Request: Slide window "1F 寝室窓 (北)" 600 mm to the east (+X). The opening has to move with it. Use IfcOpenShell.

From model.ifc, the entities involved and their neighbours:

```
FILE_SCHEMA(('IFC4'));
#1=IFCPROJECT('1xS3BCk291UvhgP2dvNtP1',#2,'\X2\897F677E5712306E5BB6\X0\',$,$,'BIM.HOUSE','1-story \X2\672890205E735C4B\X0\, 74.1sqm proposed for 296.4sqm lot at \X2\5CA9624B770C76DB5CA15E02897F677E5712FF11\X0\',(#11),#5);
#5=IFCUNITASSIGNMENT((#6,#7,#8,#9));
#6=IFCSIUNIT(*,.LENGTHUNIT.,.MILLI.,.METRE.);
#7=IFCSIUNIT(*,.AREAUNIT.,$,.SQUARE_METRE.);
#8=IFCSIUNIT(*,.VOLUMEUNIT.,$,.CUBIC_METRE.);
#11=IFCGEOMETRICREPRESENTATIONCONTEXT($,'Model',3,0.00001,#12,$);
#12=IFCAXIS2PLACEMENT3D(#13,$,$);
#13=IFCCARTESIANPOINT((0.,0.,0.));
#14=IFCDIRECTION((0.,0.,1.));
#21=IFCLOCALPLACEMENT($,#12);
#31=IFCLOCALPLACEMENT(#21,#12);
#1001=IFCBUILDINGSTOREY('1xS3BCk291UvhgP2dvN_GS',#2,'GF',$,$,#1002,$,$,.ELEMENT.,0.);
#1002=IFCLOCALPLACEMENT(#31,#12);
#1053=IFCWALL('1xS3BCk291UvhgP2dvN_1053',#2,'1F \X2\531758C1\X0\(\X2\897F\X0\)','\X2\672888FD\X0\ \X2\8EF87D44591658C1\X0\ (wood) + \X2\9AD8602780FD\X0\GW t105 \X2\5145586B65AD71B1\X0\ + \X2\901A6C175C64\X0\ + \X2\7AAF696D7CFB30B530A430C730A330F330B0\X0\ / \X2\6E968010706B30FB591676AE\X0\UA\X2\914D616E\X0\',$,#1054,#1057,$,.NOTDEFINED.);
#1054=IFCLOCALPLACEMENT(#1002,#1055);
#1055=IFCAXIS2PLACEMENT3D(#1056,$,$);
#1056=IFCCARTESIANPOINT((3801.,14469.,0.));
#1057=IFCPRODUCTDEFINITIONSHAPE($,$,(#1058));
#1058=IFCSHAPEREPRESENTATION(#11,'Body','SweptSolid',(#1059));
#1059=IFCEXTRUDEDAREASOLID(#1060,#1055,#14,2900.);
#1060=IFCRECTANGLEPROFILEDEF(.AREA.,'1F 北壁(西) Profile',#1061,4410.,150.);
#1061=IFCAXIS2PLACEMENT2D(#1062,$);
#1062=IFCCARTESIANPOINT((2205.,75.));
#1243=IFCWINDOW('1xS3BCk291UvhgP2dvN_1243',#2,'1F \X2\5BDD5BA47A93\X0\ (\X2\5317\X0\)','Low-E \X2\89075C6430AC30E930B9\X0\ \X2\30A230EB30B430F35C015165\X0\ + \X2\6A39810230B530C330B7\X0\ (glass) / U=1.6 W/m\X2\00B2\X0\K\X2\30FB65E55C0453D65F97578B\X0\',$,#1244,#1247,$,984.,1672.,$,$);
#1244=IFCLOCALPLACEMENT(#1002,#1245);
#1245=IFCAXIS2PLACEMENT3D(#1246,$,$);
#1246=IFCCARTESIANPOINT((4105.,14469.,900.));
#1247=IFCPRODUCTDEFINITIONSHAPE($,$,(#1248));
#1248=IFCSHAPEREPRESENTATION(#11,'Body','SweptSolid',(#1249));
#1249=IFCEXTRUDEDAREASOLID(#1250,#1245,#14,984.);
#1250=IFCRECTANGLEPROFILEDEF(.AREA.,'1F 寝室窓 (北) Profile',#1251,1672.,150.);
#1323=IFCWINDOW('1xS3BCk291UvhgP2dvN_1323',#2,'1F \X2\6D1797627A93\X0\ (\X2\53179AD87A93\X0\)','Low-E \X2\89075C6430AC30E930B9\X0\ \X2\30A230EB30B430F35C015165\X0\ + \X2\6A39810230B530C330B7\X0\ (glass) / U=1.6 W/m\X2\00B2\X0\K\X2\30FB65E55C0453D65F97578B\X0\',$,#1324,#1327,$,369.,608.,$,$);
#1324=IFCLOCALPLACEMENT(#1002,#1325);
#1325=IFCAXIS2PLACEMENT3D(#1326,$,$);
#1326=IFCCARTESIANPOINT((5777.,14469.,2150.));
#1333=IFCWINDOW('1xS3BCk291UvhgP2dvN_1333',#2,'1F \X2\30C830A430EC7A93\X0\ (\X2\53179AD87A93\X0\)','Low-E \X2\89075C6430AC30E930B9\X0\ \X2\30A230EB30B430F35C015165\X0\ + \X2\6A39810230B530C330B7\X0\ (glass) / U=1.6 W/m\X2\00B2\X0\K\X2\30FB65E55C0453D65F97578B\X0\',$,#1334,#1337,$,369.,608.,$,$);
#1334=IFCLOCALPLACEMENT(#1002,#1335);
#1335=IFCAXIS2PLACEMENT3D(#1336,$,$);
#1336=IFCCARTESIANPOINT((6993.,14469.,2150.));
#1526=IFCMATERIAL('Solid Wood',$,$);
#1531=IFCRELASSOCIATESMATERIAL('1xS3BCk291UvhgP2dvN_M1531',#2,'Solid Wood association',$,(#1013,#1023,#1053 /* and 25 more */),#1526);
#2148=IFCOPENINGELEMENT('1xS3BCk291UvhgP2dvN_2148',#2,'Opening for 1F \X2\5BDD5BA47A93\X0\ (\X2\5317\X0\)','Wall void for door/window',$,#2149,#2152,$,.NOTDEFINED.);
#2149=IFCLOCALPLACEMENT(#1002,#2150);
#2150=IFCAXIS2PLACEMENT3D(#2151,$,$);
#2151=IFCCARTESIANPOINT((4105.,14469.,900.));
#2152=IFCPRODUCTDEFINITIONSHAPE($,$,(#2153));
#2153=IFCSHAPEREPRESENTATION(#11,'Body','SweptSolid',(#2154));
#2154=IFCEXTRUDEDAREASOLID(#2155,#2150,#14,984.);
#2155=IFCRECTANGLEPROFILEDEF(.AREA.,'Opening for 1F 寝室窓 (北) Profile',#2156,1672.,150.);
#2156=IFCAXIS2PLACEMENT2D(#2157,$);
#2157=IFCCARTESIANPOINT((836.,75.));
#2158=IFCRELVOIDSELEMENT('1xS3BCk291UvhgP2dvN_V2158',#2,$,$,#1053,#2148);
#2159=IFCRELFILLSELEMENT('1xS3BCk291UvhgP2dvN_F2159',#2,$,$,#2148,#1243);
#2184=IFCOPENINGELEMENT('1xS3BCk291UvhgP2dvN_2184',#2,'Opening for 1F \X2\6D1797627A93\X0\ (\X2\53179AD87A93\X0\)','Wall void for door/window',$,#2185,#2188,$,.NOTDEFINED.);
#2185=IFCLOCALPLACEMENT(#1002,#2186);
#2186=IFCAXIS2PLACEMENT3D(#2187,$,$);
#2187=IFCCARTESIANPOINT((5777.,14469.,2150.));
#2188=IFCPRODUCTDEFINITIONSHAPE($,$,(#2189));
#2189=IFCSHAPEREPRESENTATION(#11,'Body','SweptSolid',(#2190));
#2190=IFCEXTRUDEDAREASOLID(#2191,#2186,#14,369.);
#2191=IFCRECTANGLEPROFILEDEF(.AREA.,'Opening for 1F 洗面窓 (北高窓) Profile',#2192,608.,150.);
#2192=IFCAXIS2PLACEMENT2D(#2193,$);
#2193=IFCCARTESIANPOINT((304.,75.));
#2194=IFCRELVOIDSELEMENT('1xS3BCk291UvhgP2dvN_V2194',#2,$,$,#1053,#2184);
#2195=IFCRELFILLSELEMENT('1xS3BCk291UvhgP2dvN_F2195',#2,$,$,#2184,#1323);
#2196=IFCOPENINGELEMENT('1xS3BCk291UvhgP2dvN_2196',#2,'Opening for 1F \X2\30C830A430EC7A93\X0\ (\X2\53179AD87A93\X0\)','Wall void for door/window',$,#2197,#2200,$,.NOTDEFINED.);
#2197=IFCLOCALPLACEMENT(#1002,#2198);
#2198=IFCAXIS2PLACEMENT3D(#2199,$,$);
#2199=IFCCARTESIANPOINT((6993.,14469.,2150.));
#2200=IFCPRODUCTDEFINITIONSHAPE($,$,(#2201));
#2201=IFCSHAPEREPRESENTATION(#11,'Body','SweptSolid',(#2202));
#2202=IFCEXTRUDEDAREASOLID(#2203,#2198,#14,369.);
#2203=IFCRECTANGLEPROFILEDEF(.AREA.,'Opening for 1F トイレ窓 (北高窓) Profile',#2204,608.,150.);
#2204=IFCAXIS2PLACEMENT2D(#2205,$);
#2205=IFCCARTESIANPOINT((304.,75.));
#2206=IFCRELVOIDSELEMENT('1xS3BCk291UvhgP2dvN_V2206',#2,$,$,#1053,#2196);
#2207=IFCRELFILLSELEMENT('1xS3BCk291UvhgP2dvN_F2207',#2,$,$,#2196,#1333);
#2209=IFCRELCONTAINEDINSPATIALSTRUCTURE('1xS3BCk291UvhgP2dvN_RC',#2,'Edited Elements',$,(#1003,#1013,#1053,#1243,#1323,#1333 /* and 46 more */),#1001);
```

```python
import ifcopenshell
import ifcopenshell.api.geometry
import ifcopenshell.util.placement
import ifcopenshell.util.unit

model = ifcopenshell.open("model.ifc")
unit_scale = ifcopenshell.util.unit.calculate_unit_scale(model)

window = model.by_id(1243)
opening = window.FillsVoids[0].RelatingOpeningElement
wall = opening.VoidsElements[0].RelatingBuildingElement

wall_matrix = ifcopenshell.util.placement.get_local_placement(wall.ObjectPlacement)
shift = wall_matrix[:3, 0] * 0.6 / unit_scale
before = ifcopenshell.util.placement.get_local_placement(window.ObjectPlacement)[:3, 3].copy()

# The window is not placed relative to its opening, so move both.
for product in (opening, window):
    matrix = ifcopenshell.util.placement.get_local_placement(product.ObjectPlacement)
    matrix[:3, 3] += shift
    ifcopenshell.api.geometry.edit_object_placement(model, product=product, matrix=matrix, is_si=False)

after = ifcopenshell.util.placement.get_local_placement(window.ObjectPlacement)[:3, 3]
print("window moved by", (after - before).round(3) + 0.0)

model.write("model-out.ifc")
```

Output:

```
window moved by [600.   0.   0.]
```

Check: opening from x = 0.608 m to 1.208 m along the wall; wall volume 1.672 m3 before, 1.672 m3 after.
